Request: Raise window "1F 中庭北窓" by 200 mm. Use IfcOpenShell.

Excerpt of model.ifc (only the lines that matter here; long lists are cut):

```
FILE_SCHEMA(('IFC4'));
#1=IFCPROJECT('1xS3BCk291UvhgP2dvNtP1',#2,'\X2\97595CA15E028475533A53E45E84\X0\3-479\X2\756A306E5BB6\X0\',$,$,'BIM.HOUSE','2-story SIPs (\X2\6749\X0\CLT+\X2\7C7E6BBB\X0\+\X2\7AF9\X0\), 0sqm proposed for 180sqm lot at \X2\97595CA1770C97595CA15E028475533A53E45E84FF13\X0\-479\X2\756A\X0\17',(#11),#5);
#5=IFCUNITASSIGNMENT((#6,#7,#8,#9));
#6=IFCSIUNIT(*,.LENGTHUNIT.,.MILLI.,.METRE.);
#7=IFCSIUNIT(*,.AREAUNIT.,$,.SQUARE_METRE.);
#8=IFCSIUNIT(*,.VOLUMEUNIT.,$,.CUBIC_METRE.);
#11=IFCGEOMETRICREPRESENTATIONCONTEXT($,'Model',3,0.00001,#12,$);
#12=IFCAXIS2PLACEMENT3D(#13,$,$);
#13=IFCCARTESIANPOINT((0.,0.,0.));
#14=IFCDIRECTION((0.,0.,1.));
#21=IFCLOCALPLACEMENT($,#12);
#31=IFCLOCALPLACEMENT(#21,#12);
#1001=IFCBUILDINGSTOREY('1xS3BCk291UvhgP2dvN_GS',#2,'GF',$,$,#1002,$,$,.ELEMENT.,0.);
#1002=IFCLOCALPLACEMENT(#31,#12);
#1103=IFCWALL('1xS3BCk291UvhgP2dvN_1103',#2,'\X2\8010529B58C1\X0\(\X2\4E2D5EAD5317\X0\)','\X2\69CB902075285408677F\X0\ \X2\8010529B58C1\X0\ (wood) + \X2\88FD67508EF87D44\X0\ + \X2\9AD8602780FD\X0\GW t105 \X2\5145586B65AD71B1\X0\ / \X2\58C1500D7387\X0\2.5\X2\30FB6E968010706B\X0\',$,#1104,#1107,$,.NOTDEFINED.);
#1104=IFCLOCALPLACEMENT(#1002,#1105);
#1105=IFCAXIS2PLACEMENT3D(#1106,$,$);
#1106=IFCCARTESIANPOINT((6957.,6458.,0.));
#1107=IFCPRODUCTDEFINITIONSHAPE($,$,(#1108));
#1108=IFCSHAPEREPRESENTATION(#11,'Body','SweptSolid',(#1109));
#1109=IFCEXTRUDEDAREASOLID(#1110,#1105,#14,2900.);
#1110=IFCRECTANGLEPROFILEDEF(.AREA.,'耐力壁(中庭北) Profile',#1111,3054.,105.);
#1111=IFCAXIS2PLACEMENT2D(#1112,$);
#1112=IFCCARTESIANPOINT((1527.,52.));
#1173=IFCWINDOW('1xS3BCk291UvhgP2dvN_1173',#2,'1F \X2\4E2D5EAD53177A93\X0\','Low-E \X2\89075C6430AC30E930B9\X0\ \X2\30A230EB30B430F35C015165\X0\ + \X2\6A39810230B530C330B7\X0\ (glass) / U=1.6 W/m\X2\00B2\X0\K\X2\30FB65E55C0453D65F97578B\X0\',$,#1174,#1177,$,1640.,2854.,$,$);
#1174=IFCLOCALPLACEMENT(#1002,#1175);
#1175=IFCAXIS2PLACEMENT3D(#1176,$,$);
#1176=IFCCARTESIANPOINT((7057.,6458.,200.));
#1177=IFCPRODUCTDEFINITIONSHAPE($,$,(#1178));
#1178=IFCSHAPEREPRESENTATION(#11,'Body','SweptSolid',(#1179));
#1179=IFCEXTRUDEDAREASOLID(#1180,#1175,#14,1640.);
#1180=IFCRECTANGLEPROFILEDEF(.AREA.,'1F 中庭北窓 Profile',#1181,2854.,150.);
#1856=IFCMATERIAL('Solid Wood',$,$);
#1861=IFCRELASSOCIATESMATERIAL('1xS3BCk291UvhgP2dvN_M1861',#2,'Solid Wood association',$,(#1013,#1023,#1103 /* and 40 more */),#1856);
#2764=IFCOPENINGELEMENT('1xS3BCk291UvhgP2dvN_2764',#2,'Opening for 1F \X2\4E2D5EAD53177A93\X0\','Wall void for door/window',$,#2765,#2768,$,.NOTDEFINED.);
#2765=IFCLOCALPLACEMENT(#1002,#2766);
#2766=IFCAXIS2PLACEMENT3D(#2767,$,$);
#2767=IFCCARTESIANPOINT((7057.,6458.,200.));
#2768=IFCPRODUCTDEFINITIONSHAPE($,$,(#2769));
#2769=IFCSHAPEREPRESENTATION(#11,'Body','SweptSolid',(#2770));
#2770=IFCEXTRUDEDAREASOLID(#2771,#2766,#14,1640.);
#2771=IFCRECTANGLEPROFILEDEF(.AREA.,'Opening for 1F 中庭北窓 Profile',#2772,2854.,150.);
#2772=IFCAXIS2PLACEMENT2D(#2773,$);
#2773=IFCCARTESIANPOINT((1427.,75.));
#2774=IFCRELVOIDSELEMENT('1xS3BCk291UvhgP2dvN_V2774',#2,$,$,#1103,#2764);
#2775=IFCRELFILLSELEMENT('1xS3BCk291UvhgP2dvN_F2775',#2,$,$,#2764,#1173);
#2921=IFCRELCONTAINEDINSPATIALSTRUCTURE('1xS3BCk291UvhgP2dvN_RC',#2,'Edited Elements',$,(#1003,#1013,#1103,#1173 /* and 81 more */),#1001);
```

```python
import numpy as np
import ifcopenshell
import ifcopenshell.api.geometry
import ifcopenshell.util.placement
import ifcopenshell.util.unit

model = ifcopenshell.open("model.ifc")
unit_scale = ifcopenshell.util.unit.calculate_unit_scale(model)

window = model.by_guid("1xS3BCk291UvhgP2dvN_1173")
opening = window.FillsVoids[0].RelatingOpeningElement
dz = 0.2 / unit_scale

shift = np.array([0.0, 0.0, dz])
# The window is not placed relative to its opening, so move both.
for product in (opening, window):
    matrix = ifcopenshell.util.placement.get_local_placement(product.ObjectPlacement)
    matrix[:3, 3] += shift
    ifcopenshell.api.geometry.edit_object_placement(model, product=product, matrix=matrix, is_si=False)

print(f"moved by {dz * unit_scale:+.3f} m")

model.write("model_updated.ifc")
```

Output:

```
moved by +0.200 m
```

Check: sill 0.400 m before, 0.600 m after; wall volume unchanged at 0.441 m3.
